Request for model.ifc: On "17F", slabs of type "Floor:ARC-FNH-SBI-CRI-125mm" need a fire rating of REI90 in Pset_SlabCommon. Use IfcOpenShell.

First a look at what the model holds.

```python
import ifcopenshell
import ifcopenshell.util.element

model = ifcopenshell.open("model.ifc")
print(model.schema)
storey = next(s for s in model.by_type("IfcBuildingStorey") if s.Name == "17F")
slabs = [e for e in ifcopenshell.util.element.get_decomposition(storey) if e.is_a("IfcSlab")]
seen = {}
for e in slabs:
    element_type = ifcopenshell.util.element.get_type(e)
    key = (element_type.Name if element_type != e and element_type else None, ifcopenshell.util.element.get_pset(e, "Pset_SlabCommon", "FireRating"))
    seen[key] = seen.get(key, 0) + 1
for (name, value), count in sorted(seen.items(), key=str):
    print(count, "x", name, "|", value)
```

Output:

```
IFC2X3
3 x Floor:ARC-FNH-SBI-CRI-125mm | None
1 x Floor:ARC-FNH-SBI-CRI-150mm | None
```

```python
import ifcopenshell
import ifcopenshell.api.pset
import ifcopenshell.util.element

model = ifcopenshell.open("model.ifc")

storey = next(s for s in model.by_type("IfcBuildingStorey") if s.Name == "17F")
slabs = [e for e in ifcopenshell.util.element.get_decomposition(storey) if e.is_a("IfcSlab")]

count = 0
for e in slabs:
    element_type = ifcopenshell.util.element.get_type(e)
    if element_type in (None, e) or element_type.Name != "Floor:ARC-FNH-SBI-CRI-125mm":
        continue
    # add_pset returns the element's existing set when there is one.
    pset = ifcopenshell.api.pset.add_pset(model, product=e, name="Pset_SlabCommon")
    ifcopenshell.api.pset.edit_pset(model, pset=pset, properties={"FireRating": "REI90"})
    count += 1

print(count, "slabs updated")

model.write("model-out.ifc")
```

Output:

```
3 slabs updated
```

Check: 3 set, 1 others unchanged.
